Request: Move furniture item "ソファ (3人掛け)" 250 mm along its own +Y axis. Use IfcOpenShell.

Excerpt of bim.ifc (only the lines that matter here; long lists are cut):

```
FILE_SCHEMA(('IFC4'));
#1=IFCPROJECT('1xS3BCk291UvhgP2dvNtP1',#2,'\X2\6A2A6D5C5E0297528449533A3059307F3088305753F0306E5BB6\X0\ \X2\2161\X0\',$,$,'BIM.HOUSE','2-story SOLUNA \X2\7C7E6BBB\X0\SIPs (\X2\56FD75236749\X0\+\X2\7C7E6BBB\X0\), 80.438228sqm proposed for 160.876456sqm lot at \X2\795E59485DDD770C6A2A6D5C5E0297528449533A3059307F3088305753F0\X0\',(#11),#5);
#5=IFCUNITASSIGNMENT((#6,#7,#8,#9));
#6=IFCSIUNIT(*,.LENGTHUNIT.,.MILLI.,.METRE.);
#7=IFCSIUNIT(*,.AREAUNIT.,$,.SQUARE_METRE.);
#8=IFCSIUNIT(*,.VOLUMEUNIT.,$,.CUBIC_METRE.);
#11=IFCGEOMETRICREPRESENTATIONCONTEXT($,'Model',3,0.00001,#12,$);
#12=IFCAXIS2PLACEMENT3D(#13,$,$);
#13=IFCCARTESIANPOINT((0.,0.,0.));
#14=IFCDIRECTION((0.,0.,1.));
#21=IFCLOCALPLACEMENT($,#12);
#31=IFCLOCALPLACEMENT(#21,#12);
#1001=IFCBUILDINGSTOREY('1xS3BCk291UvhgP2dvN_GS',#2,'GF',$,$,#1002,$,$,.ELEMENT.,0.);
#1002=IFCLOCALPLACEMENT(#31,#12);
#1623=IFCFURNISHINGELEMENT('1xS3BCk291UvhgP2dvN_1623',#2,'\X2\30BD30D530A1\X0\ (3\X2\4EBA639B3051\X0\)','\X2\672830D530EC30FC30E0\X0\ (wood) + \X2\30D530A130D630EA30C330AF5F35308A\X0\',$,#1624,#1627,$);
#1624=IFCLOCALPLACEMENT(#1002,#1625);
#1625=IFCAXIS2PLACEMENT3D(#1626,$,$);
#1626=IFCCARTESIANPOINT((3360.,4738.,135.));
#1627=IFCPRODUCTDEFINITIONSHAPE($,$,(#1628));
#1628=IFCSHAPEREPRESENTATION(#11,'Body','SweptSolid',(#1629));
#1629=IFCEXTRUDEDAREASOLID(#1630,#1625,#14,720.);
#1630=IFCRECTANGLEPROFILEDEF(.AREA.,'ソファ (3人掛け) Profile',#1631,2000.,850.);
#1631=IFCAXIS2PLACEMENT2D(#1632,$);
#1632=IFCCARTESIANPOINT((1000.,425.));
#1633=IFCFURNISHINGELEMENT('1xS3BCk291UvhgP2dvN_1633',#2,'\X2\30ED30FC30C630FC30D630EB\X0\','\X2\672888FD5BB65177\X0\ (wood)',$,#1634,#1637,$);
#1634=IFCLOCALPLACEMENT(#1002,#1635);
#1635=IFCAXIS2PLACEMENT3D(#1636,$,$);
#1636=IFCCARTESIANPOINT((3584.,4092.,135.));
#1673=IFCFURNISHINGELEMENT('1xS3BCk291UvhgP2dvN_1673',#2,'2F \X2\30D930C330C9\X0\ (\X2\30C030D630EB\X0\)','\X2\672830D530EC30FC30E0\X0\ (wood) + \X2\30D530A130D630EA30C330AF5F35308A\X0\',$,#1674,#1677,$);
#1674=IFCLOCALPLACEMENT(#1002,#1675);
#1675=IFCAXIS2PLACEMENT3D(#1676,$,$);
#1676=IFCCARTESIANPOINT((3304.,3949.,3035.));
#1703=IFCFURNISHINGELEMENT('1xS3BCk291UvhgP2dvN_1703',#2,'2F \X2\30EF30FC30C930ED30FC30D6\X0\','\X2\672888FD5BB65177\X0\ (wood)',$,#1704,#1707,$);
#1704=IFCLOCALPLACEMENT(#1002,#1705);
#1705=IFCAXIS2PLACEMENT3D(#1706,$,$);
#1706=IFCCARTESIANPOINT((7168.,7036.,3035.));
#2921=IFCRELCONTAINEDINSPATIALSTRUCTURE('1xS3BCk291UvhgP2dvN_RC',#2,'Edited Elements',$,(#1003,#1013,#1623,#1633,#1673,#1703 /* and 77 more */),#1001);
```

```python
import ifcopenshell
import ifcopenshell.api.geometry
import ifcopenshell.util.placement
import ifcopenshell.util.unit

model = ifcopenshell.open("bim.ifc")
unit_scale = ifcopenshell.util.unit.calculate_unit_scale(model)

item = model.by_id(1623)
matrix = ifcopenshell.util.placement.get_local_placement(item.ObjectPlacement)
matrix[:3, 3] += matrix[:3, 1] * 0.25 / unit_scale
ifcopenshell.api.geometry.edit_object_placement(model, product=item, matrix=matrix, is_si=False)

print(ifcopenshell.util.placement.get_local_placement(item.ObjectPlacement).round(3) + 0.0)

model.write("bim_rev.ifc")
```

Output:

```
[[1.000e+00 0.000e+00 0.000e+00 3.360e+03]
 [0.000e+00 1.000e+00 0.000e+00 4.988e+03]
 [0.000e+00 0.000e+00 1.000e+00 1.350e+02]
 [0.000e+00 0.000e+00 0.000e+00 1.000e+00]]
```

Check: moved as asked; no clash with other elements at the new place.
